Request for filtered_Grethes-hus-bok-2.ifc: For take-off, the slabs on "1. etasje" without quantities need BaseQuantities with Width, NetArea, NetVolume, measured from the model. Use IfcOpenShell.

First a look at what the model holds.

```python
import ifcopenshell
import ifcopenshell.util.element
import ifcopenshell.util.unit

model = ifcopenshell.open("filtered_Grethes-hus-bok-2.ifc")
print(model.schema)
for unit_type in ("LENGTHUNIT", "AREAUNIT", "VOLUMEUNIT"):
    print(unit_type, ifcopenshell.util.unit.calculate_unit_scale(model, unit_type))
storey = next(s for s in model.by_type("IfcBuildingStorey") if s.Name == "1. etasje")
slabs = [e for e in ifcopenshell.util.element.get_decomposition(storey) if e.is_a("IfcSlab")]
for e in sorted(slabs, key=lambda e: e.id()):
    print(e.id(), e.is_a(), e.Name, list(ifcopenshell.util.element.get_psets(e, qtos_only=True)), sep=" | ")
```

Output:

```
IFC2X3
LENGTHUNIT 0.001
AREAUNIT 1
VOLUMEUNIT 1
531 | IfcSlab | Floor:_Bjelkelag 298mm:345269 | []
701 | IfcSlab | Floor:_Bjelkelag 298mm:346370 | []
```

```python
import ifcopenshell
import ifcopenshell.api.pset
import ifcopenshell.geom
import ifcopenshell.util.element
import ifcopenshell.util.shape
import ifcopenshell.util.unit

model = ifcopenshell.open("filtered_Grethes-hus-bok-2.ifc")
unit_scale = ifcopenshell.util.unit.calculate_unit_scale(model)
area_scale = ifcopenshell.util.unit.calculate_unit_scale(model, "AREAUNIT")
volume_scale = ifcopenshell.util.unit.calculate_unit_scale(model, "VOLUMEUNIT")
settings = ifcopenshell.geom.settings()

storey = next(s for s in model.by_type("IfcBuildingStorey") if s.Name == "1. etasje")
slabs = [e for e in ifcopenshell.util.element.get_decomposition(storey) if e.is_a("IfcSlab")]

for e in sorted(slabs, key=lambda e: e.id()):
    if ifcopenshell.util.element.get_psets(e, qtos_only=True, should_inherit=False):
        continue
    # Geometry comes back in metres, in the element's own axes.
    shape = ifcopenshell.geom.create_shape(settings, e)
    values = {
        "Width": ifcopenshell.util.shape.get_z(shape.geometry) / unit_scale,
        "NetArea": ifcopenshell.util.shape.get_footprint_area(shape.geometry) / area_scale,
        "NetVolume": ifcopenshell.util.shape.get_volume(shape.geometry) / volume_scale,
    }
    qto = ifcopenshell.api.pset.add_qto(model, product=e, name="BaseQuantities")
    ifcopenshell.api.pset.edit_qto(model, qto=qto, properties=values)
    print(e.id(), {k: round(v, 3) for k, v in values.items()})

model.write("filtered_Grethes-hus-bok-2_v2.ifc")
```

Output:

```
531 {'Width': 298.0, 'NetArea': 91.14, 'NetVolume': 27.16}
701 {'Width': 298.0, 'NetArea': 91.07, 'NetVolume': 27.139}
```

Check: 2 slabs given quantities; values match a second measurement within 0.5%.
